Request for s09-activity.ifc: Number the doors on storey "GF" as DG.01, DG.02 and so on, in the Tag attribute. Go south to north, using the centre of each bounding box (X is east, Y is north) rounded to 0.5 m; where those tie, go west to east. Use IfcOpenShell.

First a look at what the model holds.

```python
import ifcopenshell
import ifcopenshell.util.element
import ifcopenshell.util.placement

model = ifcopenshell.open("s09-activity.ifc")
print(model.schema)
storey = next(s for s in model.by_type("IfcBuildingStorey") if s.Name == "GF")
doors = [e for e in ifcopenshell.util.element.get_decomposition(storey) if e.is_a("IfcDoor")]
for e in sorted(doors, key=lambda e: e.id()):
    origin = ifcopenshell.util.placement.get_local_placement(e.ObjectPlacement)[:3, 3]
    print(e.id(), e.Tag, e.Name, origin.round(2) + 0.0, sep=" | ")
```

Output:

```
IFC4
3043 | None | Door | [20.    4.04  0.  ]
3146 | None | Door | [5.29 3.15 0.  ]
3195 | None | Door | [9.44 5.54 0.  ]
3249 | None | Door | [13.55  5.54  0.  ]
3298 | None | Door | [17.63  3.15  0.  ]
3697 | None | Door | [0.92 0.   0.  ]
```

```python
import ifcopenshell
import ifcopenshell.geom
import ifcopenshell.util.element
import ifcopenshell.util.shape

model = ifcopenshell.open("s09-activity.ifc")
settings = ifcopenshell.geom.settings()
settings.set("use-world-coords", True)


def centre(element):
    shape = ifcopenshell.geom.create_shape(settings, element)
    return ifcopenshell.util.shape.get_bbox_centroid(shape.geometry)


storey = next(s for s in model.by_type("IfcBuildingStorey") if s.Name == "GF")
doors = [e for e in ifcopenshell.util.element.get_decomposition(storey) if e.is_a("IfcDoor")]

# Insertion points can sit at a corner or the storey origin, so sort by the geometry (in metres).
centres = {e: centre(e) for e in doors}
doors.sort(key=lambda e: (round(centres[e][1] / 0.5), centres[e][0]))

for i, e in enumerate(doors, start=1):
    number = f"DG.{i:02d}"
    e.Tag = number
    print(e.id(), number)

model.write("s09-activity_updated.ifc")
```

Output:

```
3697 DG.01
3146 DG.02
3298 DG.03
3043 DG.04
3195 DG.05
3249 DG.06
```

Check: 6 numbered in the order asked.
